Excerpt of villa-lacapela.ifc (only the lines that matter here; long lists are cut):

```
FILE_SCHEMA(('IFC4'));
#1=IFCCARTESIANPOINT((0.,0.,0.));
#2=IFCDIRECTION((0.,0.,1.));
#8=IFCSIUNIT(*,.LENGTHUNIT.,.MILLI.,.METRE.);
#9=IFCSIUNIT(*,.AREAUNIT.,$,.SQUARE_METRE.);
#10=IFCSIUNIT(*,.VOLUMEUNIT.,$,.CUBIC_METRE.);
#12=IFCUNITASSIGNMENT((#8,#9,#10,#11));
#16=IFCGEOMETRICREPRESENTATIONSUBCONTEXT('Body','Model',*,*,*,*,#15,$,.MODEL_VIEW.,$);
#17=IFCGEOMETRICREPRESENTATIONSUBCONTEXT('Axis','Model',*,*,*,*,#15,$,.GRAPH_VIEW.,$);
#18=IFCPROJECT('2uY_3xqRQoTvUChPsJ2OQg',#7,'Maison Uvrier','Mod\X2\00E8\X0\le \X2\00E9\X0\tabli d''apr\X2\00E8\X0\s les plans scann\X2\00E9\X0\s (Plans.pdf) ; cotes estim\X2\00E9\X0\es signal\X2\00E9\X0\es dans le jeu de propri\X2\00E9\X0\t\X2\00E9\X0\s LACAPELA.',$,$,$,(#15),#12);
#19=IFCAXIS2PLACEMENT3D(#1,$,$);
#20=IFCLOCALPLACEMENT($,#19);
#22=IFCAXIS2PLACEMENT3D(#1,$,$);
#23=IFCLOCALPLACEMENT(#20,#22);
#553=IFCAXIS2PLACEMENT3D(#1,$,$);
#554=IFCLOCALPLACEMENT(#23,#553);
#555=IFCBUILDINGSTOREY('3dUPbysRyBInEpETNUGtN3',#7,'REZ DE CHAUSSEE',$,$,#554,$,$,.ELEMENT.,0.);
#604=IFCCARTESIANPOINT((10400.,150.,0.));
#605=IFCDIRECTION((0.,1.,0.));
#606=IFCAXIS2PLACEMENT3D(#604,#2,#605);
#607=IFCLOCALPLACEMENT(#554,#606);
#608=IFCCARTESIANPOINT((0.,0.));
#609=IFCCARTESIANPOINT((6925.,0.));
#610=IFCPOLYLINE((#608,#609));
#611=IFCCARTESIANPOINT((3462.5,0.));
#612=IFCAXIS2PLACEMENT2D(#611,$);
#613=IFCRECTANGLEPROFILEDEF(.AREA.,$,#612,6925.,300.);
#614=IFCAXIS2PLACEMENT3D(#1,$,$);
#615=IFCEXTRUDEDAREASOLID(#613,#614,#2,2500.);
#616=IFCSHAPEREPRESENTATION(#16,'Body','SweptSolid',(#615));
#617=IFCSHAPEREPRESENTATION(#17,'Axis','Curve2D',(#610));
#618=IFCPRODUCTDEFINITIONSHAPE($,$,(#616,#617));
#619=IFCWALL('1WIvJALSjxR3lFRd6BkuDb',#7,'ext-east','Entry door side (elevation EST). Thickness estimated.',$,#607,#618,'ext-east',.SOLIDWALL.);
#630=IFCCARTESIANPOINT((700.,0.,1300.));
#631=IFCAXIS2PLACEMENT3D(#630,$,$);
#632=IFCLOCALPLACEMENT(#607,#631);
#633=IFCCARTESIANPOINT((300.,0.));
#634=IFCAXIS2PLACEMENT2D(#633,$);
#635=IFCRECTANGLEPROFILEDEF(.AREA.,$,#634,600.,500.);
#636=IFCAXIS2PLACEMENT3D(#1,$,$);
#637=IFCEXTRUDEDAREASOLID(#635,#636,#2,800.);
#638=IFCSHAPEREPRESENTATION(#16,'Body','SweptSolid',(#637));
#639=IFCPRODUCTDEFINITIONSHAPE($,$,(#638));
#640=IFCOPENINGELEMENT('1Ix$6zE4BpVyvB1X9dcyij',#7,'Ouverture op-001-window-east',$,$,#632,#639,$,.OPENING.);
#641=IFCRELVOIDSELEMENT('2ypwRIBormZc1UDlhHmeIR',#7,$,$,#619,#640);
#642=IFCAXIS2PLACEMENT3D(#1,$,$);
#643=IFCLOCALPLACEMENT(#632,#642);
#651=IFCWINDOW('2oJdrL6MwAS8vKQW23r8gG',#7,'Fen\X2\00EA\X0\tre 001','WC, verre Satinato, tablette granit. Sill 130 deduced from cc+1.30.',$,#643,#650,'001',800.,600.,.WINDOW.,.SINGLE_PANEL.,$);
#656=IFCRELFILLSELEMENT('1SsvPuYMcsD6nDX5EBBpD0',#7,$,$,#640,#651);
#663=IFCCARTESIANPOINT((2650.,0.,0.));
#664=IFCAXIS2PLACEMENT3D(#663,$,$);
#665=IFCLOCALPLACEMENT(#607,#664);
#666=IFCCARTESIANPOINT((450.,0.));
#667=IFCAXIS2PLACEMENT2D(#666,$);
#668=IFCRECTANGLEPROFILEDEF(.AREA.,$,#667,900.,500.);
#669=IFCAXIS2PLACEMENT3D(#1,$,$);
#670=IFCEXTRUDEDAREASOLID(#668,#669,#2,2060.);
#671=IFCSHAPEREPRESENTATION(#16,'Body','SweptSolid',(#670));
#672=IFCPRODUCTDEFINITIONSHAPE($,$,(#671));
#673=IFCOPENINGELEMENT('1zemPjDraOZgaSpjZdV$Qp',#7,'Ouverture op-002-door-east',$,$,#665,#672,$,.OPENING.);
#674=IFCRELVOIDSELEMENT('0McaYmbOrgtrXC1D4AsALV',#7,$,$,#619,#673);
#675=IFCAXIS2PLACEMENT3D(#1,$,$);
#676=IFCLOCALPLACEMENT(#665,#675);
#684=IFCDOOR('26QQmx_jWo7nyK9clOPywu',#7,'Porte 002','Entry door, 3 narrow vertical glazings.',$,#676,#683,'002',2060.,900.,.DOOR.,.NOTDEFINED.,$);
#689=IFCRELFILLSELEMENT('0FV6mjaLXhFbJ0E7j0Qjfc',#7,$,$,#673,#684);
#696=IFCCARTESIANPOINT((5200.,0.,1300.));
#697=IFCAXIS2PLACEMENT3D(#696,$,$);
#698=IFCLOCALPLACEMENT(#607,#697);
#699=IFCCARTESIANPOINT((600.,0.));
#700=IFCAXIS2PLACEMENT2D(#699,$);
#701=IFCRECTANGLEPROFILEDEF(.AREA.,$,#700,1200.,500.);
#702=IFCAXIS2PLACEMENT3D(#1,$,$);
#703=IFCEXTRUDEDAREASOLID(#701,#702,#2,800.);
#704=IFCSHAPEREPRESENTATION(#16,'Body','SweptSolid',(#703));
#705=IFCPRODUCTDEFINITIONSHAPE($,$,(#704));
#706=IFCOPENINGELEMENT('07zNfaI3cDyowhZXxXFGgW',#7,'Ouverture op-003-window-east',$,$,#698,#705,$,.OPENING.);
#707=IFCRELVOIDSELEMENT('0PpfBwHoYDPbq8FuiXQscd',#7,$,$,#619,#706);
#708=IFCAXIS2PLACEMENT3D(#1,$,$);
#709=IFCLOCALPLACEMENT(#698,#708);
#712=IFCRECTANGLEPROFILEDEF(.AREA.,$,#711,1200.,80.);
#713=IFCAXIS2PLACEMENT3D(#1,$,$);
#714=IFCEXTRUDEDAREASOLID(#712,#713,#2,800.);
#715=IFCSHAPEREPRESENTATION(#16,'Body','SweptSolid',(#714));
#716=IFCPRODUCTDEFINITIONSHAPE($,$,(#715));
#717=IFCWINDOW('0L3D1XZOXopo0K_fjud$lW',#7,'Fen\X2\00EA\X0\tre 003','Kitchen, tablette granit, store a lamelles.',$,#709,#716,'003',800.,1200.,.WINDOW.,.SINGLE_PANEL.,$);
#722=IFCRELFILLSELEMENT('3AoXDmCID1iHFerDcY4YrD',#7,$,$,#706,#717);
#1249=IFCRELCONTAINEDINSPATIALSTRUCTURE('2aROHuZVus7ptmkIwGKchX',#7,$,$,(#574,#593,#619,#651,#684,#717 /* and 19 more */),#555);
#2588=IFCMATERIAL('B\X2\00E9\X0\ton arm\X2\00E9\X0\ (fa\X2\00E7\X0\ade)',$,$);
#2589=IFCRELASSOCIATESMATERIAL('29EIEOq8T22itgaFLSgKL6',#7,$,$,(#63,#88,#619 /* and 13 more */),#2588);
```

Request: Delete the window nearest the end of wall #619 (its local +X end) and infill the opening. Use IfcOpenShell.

```python
import ifcopenshell
import ifcopenshell.api.feature
import ifcopenshell.api.root
import ifcopenshell.geom
import ifcopenshell.util.shape

model = ifcopenshell.open("villa-lacapela.ifc")
settings = ifcopenshell.geom.settings()


def volume(element):
    """Net volume in cubic metres, openings subtracted."""
    shape = ifcopenshell.geom.create_shape(settings, element)
    return ifcopenshell.util.shape.get_volume(shape.geometry)


window = model.by_id(717)
opening = window.FillsVoids[0].RelatingOpeningElement
wall = opening.VoidsElements[0].RelatingBuildingElement
before = volume(wall)

ifcopenshell.api.root.remove_product(model, product=window)
ifcopenshell.api.feature.remove_feature(model, feature=opening)

after = volume(wall)

print(f"wall volume {before:.3f} -> {after:.3f} m3")

model.write("villa-lacapela_v2.ifc")
```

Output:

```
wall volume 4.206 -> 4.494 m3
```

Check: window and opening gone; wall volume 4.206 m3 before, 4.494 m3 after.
